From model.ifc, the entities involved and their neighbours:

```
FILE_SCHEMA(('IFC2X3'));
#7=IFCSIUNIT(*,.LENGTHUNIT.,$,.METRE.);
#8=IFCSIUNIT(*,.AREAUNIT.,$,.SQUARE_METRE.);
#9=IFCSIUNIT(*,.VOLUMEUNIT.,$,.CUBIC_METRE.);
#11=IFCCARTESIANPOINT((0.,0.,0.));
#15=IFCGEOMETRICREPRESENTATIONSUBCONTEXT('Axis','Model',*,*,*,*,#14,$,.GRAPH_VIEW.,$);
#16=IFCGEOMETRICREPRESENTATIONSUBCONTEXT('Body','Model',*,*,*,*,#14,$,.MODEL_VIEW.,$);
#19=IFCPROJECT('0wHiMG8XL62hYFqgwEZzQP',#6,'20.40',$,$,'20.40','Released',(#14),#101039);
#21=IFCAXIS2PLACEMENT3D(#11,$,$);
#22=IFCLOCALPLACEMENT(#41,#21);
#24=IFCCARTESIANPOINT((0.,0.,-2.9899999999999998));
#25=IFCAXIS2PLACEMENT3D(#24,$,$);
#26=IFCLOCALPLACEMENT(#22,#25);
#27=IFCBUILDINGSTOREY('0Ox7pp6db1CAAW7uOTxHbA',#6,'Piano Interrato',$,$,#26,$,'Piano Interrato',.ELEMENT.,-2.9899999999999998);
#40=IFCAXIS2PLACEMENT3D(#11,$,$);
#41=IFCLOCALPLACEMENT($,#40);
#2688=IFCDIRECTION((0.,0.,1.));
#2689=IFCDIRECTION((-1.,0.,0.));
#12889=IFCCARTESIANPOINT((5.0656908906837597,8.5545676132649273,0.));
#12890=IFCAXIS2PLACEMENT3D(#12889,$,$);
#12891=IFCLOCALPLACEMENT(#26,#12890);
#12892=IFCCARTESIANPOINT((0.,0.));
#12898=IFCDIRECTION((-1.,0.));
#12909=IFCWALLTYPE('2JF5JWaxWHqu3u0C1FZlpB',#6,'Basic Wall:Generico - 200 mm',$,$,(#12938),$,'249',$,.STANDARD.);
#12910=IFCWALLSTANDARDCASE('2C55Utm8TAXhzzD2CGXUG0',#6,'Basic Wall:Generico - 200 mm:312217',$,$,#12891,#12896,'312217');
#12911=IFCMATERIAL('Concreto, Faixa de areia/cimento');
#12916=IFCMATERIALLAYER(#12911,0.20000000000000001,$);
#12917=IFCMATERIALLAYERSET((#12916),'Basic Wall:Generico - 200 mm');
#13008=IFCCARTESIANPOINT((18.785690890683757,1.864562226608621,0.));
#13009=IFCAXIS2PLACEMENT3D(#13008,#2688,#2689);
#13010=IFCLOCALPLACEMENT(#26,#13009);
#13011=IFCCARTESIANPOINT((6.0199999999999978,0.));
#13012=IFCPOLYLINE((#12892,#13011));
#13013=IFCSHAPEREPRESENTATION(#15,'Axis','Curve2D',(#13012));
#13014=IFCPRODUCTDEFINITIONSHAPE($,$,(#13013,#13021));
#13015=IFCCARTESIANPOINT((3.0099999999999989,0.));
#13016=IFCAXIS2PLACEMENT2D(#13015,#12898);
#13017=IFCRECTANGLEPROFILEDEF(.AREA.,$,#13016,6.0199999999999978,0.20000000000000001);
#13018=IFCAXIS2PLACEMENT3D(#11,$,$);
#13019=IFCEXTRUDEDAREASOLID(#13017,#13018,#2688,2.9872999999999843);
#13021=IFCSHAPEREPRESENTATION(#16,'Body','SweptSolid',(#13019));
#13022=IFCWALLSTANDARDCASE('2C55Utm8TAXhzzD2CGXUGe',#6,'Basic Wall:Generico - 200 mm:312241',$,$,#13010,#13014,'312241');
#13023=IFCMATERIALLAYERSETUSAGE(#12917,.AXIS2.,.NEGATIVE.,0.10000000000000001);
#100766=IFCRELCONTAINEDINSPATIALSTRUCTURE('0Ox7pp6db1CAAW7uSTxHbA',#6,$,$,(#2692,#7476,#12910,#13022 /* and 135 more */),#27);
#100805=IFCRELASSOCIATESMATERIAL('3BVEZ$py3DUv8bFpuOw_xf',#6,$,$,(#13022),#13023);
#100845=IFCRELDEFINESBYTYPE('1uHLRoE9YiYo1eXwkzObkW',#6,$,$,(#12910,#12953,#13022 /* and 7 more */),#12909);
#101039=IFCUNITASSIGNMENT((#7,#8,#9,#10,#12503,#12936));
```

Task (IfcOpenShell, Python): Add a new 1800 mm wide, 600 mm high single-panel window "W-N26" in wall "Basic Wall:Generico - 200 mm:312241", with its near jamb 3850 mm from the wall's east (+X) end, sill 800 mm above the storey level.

```python
import numpy as np
import ifcopenshell
import ifcopenshell.api.feature
import ifcopenshell.api.geometry
import ifcopenshell.api.root
import ifcopenshell.api.spatial
import ifcopenshell.api.type
import ifcopenshell.geom
import ifcopenshell.util.element
import ifcopenshell.util.placement
import ifcopenshell.util.representation
import ifcopenshell.util.shape
import ifcopenshell.util.unit

model = ifcopenshell.open("model.ifc")
unit_scale = ifcopenshell.util.unit.calculate_unit_scale(model)
settings = ifcopenshell.geom.settings()


def volume(element):
    """Net volume in cubic metres, openings subtracted."""
    shape = ifcopenshell.geom.create_shape(settings, element)
    return ifcopenshell.util.shape.get_volume(shape.geometry)


wall = model.by_guid("2C55Utm8TAXhzzD2CGXUGe")
storey = ifcopenshell.util.element.get_container(wall, ifc_class="IfcBuildingStorey")
context = ifcopenshell.util.representation.get_context(model, "Model", "Body", "MODEL_VIEW")
before = volume(wall)

width, height, from_end, sill = 1.8, 0.6, 3.85, 0.8  # metres

# The wall runs along its own X axis, and the end named is its -X end.
wall_shape = ifcopenshell.geom.create_shape(settings, wall)
x, y, z = ifcopenshell.util.shape.get_vertices(wall_shape.geometry).T
start = x.min() + from_end
face, thickness = float(y.min()), float(y.max() - y.min())
wall_matrix = ifcopenshell.util.placement.get_local_placement(wall.ObjectPlacement)
level = ifcopenshell.util.placement.get_local_placement(storey.ObjectPlacement)[2, 3]


def in_wall(x, y):
    """Placement at x, y metres in the wall's axes, at sill height."""
    matrix = wall_matrix.copy()
    matrix[:, 3] = wall_matrix @ np.array([x / unit_scale, y / unit_scale, 0.0, 1.0])
    matrix[2, 3] = level + sill / unit_scale
    return matrix


# Opening: a box that overshoots both wall faces by 50 mm.
opening = ifcopenshell.api.root.create_entity(model, ifc_class="IfcOpeningElement")
box = ifcopenshell.api.geometry.add_wall_representation(
    model, context=context, length=width, height=height, thickness=thickness + 0.1
)
ifcopenshell.api.geometry.assign_representation(model, product=opening, representation=box)
ifcopenshell.api.geometry.edit_object_placement(model, product=opening, matrix=in_wall(start, face - 0.05), is_si=False)
ifcopenshell.api.feature.add_feature(model, feature=opening, element=wall)

window = ifcopenshell.api.root.create_entity(model, ifc_class="IfcWindow", name="W-N26")
window.OverallWidth, window.OverallHeight = width / unit_scale, height / unit_scale
body = ifcopenshell.api.geometry.add_window_representation(
    model,
    context=context,
    overall_width=window.OverallWidth,
    overall_height=window.OverallHeight,
    partition_type="SINGLE_PANEL",
)
ifcopenshell.api.geometry.assign_representation(model, product=window, representation=body)
ifcopenshell.api.spatial.assign_container(model, products=[window], relating_structure=storey)
fills = ifcopenshell.api.feature.add_filling(model, opening=opening, element=window)
fills.OwnerHistory = window.OwnerHistory  # required in IFC2X3

# IFC2X3 keeps the operation on the window style.
style = ifcopenshell.api.root.create_entity(model, ifc_class="IfcWindowStyle", name="W-N26")
style.OperationType, style.ConstructionType = "SINGLE_PANEL", "NOTDEFINED"
style.ParameterTakesPrecedence = style.Sizeable = False
ifcopenshell.api.type.assign_type(model, related_objects=[window], relating_type=style)

# Centre the window in the wall's thickness.
ifcopenshell.api.geometry.edit_object_placement(model, product=window, matrix=in_wall(start, face), is_si=False)
window_shape = ifcopenshell.geom.create_shape(settings, window)
depth = ifcopenshell.util.shape.get_vertices(window_shape.geometry)[:, 1]
offset = face + thickness / 2 - (depth.min() + depth.max()) / 2
ifcopenshell.api.geometry.edit_object_placement(model, product=window, matrix=in_wall(start, offset), is_si=False)

after = volume(wall)

print(f"wall volume {before:.3f} -> {after:.3f} m3")

model.write("model_rev.ifc")
```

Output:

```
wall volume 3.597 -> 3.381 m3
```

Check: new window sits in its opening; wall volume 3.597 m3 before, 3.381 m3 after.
